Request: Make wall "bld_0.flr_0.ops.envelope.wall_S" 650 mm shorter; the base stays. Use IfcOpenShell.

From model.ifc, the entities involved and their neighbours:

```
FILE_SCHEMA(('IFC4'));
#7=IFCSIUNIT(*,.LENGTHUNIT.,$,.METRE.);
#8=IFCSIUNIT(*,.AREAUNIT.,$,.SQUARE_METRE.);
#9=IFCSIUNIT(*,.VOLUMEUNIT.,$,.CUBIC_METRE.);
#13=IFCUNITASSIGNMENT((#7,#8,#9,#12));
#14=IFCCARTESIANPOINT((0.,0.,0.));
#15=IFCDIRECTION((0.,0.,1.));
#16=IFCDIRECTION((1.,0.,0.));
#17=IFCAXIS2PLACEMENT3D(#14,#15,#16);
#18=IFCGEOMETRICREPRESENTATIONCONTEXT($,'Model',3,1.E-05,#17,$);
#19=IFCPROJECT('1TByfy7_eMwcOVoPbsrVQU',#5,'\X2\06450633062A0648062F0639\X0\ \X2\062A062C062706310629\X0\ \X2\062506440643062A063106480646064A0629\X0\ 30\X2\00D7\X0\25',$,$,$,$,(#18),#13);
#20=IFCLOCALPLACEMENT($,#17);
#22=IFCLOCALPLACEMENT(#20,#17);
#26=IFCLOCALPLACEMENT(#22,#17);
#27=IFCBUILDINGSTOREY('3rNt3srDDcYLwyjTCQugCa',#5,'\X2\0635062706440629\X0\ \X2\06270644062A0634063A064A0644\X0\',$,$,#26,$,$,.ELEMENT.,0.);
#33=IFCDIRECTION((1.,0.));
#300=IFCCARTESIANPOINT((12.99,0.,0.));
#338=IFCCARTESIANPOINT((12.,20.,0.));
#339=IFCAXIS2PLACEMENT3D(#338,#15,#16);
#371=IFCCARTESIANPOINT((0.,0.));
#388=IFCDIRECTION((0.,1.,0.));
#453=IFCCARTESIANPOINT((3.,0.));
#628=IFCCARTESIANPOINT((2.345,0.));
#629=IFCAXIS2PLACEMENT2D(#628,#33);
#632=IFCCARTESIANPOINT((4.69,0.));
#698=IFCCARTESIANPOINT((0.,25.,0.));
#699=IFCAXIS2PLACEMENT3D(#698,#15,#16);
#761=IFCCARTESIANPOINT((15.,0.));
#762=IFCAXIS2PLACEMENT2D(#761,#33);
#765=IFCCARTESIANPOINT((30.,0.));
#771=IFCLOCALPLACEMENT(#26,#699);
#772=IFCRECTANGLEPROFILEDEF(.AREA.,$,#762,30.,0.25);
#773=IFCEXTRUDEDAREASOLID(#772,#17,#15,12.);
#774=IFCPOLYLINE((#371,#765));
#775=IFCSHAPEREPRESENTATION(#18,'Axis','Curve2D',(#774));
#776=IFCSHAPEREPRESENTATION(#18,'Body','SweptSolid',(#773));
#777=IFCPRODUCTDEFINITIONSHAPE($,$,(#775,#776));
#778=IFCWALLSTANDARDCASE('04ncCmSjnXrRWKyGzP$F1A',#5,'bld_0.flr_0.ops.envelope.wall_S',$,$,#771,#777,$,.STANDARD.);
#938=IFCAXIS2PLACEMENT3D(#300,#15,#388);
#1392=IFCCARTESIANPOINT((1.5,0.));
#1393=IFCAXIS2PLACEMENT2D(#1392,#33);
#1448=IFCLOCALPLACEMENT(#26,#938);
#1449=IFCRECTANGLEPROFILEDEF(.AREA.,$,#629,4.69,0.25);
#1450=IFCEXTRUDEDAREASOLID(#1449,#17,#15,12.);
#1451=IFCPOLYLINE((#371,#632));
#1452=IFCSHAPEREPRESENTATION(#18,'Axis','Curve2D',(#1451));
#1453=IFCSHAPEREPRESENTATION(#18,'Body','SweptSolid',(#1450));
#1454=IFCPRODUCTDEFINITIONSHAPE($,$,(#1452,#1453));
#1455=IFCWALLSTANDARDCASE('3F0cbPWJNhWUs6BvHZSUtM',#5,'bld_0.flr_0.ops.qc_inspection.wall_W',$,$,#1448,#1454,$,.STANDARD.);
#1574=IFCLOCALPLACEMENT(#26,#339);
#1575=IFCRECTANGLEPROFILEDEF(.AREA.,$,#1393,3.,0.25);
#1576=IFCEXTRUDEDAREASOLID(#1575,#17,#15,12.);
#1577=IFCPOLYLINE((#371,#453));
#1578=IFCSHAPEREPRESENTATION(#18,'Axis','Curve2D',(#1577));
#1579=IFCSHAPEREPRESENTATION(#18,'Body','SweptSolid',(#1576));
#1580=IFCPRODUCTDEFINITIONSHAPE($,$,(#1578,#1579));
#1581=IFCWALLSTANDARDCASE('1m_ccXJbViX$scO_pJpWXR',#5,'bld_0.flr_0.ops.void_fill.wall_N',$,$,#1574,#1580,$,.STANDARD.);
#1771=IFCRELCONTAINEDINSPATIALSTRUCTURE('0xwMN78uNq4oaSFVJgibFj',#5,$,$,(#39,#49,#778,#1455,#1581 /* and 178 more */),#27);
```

```python
import ifcopenshell
import ifcopenshell.geom
import ifcopenshell.util.shape

model = ifcopenshell.open("model.ifc")
settings = ifcopenshell.geom.settings()


def volume(element):
    """Net volume in cubic metres, openings subtracted."""
    shape = ifcopenshell.geom.create_shape(settings, element)
    return ifcopenshell.util.shape.get_volume(shape.geometry)


wall = model.by_guid("04ncCmSjnXrRWKyGzP$F1A")
before = volume(wall)

body = next(r for r in wall.Representation.Representations if r.RepresentationIdentifier == "Body")
solid = body.Items[0]
old_height = solid.Depth
solid.Depth -= 0.65
after = volume(wall)

print(f"height {old_height:g} -> {solid.Depth:g}, volume {before:.3f} -> {after:.3f} m3")

model.write("model_edited.ifc")
```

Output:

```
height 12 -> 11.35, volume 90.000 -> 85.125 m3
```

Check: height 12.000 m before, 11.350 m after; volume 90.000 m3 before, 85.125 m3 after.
